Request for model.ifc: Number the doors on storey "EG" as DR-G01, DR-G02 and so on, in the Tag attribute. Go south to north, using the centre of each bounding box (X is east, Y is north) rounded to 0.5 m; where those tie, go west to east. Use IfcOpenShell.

First a look at what the model holds.

```python
import ifcopenshell
import ifcopenshell.util.element
import ifcopenshell.util.placement

model = ifcopenshell.open("model.ifc")
print(model.schema)
storey = next(s for s in model.by_type("IfcBuildingStorey") if s.Name == "EG")
doors = [e for e in ifcopenshell.util.element.get_decomposition(storey) if e.is_a("IfcDoor")]
for e in sorted(doors, key=lambda e: e.id()):
    origin = ifcopenshell.util.placement.get_local_placement(e.ObjectPlacement)[:3, 3]
    print(e.id(), e.Tag, e.Name, origin.round(2) + 0.0, sep=" | ")
```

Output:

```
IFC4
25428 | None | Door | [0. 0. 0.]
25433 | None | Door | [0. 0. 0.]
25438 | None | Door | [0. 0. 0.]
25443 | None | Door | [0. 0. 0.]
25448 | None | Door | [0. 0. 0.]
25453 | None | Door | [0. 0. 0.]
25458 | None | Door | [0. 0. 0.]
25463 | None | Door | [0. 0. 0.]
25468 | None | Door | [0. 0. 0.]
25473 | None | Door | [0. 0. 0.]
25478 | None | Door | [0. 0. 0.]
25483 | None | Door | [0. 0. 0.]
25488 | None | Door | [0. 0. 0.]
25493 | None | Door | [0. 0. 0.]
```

```python
import ifcopenshell
import ifcopenshell.geom
import ifcopenshell.util.element
import ifcopenshell.util.shape

model = ifcopenshell.open("model.ifc")
settings = ifcopenshell.geom.settings()
settings.set("use-world-coords", True)


def centre(element):
    shape = ifcopenshell.geom.create_shape(settings, element)
    return ifcopenshell.util.shape.get_bbox_centroid(shape.geometry)


storey = next(s for s in model.by_type("IfcBuildingStorey") if s.Name == "EG")
doors = [e for e in ifcopenshell.util.element.get_decomposition(storey) if e.is_a("IfcDoor")]

# Insertion points can sit at a corner or the storey origin, so sort by the geometry (in metres).
centres = {e: centre(e) for e in doors}
doors.sort(key=lambda e: (round(centres[e][1] / 0.5), centres[e][0]))

for i, e in enumerate(doors, start=1):
    number = f"DR-G{i:02d}"
    e.Tag = number
    print(e.id(), number)

model.write("model-out.ifc")
```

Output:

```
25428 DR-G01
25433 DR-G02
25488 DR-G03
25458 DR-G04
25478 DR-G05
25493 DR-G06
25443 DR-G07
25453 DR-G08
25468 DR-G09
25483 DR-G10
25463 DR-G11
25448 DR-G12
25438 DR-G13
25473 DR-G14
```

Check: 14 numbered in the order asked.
